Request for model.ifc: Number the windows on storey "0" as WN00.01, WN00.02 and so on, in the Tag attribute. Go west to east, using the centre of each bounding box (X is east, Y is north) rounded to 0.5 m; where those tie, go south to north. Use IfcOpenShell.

First a look at what the model holds.

```python
import ifcopenshell
import ifcopenshell.util.element
import ifcopenshell.util.placement

model = ifcopenshell.open("model.ifc")
print(model.schema)
storey = next(s for s in model.by_type("IfcBuildingStorey") if s.Name == "0")
windows = [e for e in ifcopenshell.util.element.get_decomposition(storey) if e.is_a("IfcWindow")]
for e in sorted(windows, key=lambda e: e.id()):
    origin = ifcopenshell.util.placement.get_local_placement(e.ObjectPlacement)[:3, 3]
    print(e.id(), e.Tag, e.Name, origin.round(2) + 0.0, sep=" | ")
```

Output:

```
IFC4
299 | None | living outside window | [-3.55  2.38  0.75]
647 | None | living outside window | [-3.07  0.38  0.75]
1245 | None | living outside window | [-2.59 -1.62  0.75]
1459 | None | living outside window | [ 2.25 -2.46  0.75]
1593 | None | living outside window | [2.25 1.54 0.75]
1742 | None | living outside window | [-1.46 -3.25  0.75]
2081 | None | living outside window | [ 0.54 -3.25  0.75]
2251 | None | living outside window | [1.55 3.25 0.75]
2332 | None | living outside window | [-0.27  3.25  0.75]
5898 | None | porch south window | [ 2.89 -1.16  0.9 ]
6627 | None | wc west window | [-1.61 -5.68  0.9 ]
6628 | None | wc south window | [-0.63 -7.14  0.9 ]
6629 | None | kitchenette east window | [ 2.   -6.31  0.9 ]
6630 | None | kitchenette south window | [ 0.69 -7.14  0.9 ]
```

```python
import ifcopenshell
import ifcopenshell.geom
import ifcopenshell.util.element
import ifcopenshell.util.shape

model = ifcopenshell.open("model.ifc")
settings = ifcopenshell.geom.settings()
settings.set("use-world-coords", True)


def centre(element):
    shape = ifcopenshell.geom.create_shape(settings, element)
    return ifcopenshell.util.shape.get_bbox_centroid(shape.geometry)


storey = next(s for s in model.by_type("IfcBuildingStorey") if s.Name == "0")
windows = [e for e in ifcopenshell.util.element.get_decomposition(storey) if e.is_a("IfcWindow")]

# Insertion points can sit at a corner or the storey origin, so sort by the geometry (in metres).
centres = {e: centre(e) for e in windows}
windows.sort(key=lambda e: (round(centres[e][0] / 0.5), centres[e][1]))

for i, e in enumerate(windows, start=1):
    number = f"WN00.{i:02d}"
    e.Tag = number
    print(e.id(), number)

model.write("model_v2.ifc")
```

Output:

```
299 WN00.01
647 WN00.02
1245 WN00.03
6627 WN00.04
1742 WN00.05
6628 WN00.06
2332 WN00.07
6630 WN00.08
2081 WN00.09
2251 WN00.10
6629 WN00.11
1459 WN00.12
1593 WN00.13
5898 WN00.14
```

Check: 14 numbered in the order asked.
